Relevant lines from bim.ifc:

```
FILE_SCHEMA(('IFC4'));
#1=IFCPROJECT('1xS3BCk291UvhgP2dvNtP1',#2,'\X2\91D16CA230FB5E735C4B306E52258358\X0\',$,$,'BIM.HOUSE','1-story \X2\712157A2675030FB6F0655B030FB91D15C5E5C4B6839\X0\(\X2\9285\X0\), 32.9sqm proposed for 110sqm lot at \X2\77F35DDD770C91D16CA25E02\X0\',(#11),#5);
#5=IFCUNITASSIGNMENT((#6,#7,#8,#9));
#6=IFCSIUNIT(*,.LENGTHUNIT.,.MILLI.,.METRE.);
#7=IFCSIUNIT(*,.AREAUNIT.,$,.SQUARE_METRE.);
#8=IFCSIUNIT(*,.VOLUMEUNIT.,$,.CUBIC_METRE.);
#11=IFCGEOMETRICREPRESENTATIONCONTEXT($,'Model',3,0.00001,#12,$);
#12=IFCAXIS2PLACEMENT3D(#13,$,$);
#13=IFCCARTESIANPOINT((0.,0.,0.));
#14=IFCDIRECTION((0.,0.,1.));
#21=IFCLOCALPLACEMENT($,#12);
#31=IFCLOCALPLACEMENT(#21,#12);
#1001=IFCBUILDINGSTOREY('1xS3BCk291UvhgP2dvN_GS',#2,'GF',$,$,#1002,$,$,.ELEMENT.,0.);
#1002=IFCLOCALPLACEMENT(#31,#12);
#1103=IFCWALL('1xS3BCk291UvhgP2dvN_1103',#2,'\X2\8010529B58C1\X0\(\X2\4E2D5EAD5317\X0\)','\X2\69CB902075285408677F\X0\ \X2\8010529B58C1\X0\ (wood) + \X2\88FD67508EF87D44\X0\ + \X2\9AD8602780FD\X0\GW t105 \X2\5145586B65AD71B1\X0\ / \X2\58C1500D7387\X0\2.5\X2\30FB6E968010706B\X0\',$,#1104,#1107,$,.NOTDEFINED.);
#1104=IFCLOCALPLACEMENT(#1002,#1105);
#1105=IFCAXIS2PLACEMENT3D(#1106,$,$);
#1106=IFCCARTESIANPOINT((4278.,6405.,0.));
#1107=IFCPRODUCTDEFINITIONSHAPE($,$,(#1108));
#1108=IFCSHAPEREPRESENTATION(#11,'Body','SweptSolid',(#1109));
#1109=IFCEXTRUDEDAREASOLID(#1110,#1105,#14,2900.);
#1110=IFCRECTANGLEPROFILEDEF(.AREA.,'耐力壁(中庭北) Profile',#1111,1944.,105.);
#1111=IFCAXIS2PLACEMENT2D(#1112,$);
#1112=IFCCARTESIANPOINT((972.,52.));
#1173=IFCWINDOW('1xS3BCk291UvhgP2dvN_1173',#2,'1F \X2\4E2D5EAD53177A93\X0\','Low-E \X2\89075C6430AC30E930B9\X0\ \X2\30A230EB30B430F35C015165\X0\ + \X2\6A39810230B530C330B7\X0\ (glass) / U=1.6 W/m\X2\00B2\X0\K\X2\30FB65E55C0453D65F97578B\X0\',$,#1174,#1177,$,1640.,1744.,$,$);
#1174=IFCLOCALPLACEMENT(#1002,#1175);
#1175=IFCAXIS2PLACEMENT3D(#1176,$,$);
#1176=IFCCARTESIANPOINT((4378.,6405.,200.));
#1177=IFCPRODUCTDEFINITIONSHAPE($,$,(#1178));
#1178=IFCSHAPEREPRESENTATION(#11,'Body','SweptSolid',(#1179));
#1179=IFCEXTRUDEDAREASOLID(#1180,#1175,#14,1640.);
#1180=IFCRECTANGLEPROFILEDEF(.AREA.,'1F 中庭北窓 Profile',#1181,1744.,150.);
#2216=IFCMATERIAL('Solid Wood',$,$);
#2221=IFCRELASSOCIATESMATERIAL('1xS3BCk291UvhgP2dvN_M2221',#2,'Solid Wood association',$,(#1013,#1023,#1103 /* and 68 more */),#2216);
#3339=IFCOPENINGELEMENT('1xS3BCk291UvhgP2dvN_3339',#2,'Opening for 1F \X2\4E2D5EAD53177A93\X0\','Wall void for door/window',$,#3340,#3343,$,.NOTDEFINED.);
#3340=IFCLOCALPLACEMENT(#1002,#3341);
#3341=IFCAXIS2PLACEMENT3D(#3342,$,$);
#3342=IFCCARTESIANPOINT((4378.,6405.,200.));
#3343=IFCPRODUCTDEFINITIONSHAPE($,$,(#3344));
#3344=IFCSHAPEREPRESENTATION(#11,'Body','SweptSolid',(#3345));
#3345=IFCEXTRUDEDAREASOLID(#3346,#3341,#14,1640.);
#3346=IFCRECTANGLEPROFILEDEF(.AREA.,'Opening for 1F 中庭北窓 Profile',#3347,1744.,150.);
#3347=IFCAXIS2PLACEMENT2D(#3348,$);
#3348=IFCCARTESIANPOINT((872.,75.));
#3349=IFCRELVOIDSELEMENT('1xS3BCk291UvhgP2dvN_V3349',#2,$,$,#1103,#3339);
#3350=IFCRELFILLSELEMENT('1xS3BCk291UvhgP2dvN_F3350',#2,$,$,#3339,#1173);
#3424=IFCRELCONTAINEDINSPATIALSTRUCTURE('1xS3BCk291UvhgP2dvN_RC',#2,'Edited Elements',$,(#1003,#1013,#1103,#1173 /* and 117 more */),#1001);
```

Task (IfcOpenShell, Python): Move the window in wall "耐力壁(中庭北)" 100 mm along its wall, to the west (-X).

```python
import ifcopenshell
import ifcopenshell.api.geometry
import ifcopenshell.util.placement
import ifcopenshell.util.unit

model = ifcopenshell.open("bim.ifc")
unit_scale = ifcopenshell.util.unit.calculate_unit_scale(model)

window = model.by_id(1173)
opening = window.FillsVoids[0].RelatingOpeningElement
wall = opening.VoidsElements[0].RelatingBuildingElement

wall_matrix = ifcopenshell.util.placement.get_local_placement(wall.ObjectPlacement)
shift = wall_matrix[:3, 0] * -0.1 / unit_scale
before = ifcopenshell.util.placement.get_local_placement(window.ObjectPlacement)[:3, 3].copy()

# The window is not placed relative to its opening, so move both.
for product in (opening, window):
    matrix = ifcopenshell.util.placement.get_local_placement(product.ObjectPlacement)
    matrix[:3, 3] += shift
    ifcopenshell.api.geometry.edit_object_placement(model, product=product, matrix=matrix, is_si=False)

after = ifcopenshell.util.placement.get_local_placement(window.ObjectPlacement)[:3, 3]
print("window moved by", (after - before).round(3) + 0.0)

model.write("bim_edited.ifc")
```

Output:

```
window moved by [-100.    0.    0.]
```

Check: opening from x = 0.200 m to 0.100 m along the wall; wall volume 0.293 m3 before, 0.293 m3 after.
